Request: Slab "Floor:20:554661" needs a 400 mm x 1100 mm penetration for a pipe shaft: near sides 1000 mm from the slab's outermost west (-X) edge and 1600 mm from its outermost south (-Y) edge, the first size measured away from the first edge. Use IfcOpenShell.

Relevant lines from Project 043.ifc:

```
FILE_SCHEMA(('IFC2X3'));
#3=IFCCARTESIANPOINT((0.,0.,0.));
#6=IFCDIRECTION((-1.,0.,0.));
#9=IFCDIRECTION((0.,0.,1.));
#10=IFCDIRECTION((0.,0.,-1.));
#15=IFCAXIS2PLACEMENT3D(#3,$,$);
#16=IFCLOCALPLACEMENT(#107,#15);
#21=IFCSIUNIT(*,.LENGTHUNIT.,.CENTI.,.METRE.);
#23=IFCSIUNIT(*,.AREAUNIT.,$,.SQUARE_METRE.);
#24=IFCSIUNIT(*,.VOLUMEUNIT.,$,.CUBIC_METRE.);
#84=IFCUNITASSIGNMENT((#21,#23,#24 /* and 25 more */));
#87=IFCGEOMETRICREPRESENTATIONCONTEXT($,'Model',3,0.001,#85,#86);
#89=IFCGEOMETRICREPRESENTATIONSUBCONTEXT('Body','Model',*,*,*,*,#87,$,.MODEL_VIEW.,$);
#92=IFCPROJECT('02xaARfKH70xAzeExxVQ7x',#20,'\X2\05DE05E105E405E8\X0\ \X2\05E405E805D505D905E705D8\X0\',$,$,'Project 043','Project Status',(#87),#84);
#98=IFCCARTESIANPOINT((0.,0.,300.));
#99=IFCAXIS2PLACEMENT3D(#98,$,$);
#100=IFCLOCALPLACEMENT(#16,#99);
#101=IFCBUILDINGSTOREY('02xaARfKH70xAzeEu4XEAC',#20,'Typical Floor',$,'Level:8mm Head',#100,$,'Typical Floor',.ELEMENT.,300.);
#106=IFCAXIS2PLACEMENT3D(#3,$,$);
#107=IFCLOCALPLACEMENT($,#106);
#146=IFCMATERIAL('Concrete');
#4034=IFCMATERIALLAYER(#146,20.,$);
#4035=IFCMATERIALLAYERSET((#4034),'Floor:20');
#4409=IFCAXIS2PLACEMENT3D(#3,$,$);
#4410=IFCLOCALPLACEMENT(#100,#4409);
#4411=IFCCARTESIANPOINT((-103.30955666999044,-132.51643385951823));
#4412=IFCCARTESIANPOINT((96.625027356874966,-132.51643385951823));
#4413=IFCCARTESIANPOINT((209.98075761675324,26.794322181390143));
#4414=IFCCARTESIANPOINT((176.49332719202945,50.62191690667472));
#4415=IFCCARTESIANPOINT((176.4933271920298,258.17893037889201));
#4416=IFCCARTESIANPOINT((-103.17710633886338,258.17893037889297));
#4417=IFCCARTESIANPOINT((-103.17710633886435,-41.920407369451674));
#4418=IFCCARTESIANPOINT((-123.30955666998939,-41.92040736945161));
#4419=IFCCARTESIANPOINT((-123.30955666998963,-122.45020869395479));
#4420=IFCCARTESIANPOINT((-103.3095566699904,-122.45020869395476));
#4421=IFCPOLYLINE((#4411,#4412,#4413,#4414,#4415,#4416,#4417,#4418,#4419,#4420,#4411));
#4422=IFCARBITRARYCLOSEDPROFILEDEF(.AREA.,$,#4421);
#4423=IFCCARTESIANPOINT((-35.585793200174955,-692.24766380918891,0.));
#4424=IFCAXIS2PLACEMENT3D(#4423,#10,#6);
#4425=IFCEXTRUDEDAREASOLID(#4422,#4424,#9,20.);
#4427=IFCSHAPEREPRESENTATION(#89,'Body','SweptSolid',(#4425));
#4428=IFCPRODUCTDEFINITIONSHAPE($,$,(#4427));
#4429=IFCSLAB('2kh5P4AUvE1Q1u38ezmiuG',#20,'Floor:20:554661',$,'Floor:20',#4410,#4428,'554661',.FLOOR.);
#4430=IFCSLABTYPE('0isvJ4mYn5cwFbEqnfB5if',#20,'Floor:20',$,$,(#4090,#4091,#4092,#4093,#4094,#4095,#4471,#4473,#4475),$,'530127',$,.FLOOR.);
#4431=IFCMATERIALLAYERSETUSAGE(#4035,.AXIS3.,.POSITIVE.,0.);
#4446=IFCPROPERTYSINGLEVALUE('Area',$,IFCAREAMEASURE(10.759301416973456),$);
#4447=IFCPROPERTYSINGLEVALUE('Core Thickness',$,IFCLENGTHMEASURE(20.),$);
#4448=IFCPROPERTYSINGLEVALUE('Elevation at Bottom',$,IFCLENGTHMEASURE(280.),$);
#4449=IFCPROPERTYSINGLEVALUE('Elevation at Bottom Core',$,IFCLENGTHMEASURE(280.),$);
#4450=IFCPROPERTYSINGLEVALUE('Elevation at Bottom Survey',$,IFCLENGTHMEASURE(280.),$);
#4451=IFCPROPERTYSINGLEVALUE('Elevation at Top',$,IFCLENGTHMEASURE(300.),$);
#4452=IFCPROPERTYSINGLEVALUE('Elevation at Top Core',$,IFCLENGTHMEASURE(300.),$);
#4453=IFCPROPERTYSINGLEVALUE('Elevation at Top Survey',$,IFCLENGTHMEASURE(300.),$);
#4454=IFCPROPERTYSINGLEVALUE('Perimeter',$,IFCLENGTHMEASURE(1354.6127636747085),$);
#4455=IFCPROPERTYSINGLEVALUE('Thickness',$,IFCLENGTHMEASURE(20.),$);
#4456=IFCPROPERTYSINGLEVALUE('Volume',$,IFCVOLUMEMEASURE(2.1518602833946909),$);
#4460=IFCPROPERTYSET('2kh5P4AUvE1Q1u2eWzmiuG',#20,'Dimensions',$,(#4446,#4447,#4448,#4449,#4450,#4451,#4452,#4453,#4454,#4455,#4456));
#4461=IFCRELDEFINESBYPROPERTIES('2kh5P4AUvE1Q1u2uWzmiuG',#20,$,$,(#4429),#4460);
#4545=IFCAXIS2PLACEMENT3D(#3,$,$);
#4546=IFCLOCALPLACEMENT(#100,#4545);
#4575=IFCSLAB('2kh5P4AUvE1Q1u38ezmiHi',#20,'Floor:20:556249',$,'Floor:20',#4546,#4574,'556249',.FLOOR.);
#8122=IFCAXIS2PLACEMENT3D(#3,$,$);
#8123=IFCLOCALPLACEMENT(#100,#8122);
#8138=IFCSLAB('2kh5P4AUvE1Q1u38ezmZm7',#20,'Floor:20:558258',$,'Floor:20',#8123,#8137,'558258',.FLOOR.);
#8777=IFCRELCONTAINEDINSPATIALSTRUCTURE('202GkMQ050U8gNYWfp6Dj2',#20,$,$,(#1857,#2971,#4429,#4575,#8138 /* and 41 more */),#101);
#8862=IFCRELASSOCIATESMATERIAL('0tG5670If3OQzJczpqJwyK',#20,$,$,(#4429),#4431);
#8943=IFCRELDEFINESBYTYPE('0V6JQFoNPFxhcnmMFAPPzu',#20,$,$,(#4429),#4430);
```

```python
import numpy as np
import ifcopenshell
import ifcopenshell.api.feature
import ifcopenshell.api.geometry
import ifcopenshell.api.pset
import ifcopenshell.api.root
import ifcopenshell.geom
import ifcopenshell.util.element
import ifcopenshell.util.placement
import ifcopenshell.util.representation
import ifcopenshell.util.shape
import ifcopenshell.util.unit

model = ifcopenshell.open("Project 043.ifc")
unit_scale = ifcopenshell.util.unit.calculate_unit_scale(model)
area_scale = ifcopenshell.util.unit.calculate_unit_scale(model, "AREAUNIT")
volume_scale = ifcopenshell.util.unit.calculate_unit_scale(model, "VOLUMEUNIT")
settings = ifcopenshell.geom.settings()


def volume(element):
    """Net volume in cubic metres, openings subtracted."""
    shape = ifcopenshell.geom.create_shape(settings, element)
    return ifcopenshell.util.shape.get_volume(shape.geometry)


slab = model.by_guid("2kh5P4AUvE1Q1u38ezmiuG")
before = volume(slab)

# Extent in the slab's own axes, in metres. The edges named are its -X and -Y sides.
slab_shape = ifcopenshell.geom.create_shape(settings, slab)
vertices = ifcopenshell.util.shape.get_vertices(slab_shape.geometry)
x_min, y_min, bottom = vertices.min(axis=0)
top = vertices[:, 2].max()

opening = ifcopenshell.api.root.create_entity(model, ifc_class="IfcOpeningElement", name="Pipe shaft opening")
context = ifcopenshell.util.representation.get_context(model, "Model", "Body", "MODEL_VIEW")
width, depth = 0.4, 1.1
outline = [(0.0, 0.0), (width, 0.0), (width, depth), (0.0, depth), (0.0, 0.0)]
# Overshoot both faces by 50 mm so the cut is clean.
shape = ifcopenshell.api.geometry.add_slab_representation(
    model, context=context, depth=top - bottom + 0.1, polyline=outline
)
ifcopenshell.api.geometry.assign_representation(model, product=opening, representation=shape)

matrix = ifcopenshell.util.placement.get_local_placement(slab.ObjectPlacement)
matrix[:, 3] = matrix @ np.append(np.array([x_min + 1, y_min + 1.6, bottom - 0.05]) / unit_scale, 1.0)
ifcopenshell.api.geometry.edit_object_placement(model, product=opening, matrix=matrix, is_si=False)
ifcopenshell.api.feature.add_feature(model, feature=opening, element=slab)

after = volume(slab)

# Update the slab's stored quantities.
pset = model.by_id(ifcopenshell.util.element.get_pset(slab, "Dimensions", should_inherit=False)["id"])
ifcopenshell.api.pset.edit_pset(model, pset=pset, properties={
    "Area": model.create_entity("IfcAreaMeasure", after / (top - bottom) / area_scale),
    "Volume": model.create_entity("IfcVolumeMeasure", after / volume_scale),
})

print(f"slab volume {before:.3f} -> {after:.3f} m3")

model.write("Project 043_edited.ifc")
```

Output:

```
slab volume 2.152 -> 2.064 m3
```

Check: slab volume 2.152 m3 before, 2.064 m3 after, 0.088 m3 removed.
